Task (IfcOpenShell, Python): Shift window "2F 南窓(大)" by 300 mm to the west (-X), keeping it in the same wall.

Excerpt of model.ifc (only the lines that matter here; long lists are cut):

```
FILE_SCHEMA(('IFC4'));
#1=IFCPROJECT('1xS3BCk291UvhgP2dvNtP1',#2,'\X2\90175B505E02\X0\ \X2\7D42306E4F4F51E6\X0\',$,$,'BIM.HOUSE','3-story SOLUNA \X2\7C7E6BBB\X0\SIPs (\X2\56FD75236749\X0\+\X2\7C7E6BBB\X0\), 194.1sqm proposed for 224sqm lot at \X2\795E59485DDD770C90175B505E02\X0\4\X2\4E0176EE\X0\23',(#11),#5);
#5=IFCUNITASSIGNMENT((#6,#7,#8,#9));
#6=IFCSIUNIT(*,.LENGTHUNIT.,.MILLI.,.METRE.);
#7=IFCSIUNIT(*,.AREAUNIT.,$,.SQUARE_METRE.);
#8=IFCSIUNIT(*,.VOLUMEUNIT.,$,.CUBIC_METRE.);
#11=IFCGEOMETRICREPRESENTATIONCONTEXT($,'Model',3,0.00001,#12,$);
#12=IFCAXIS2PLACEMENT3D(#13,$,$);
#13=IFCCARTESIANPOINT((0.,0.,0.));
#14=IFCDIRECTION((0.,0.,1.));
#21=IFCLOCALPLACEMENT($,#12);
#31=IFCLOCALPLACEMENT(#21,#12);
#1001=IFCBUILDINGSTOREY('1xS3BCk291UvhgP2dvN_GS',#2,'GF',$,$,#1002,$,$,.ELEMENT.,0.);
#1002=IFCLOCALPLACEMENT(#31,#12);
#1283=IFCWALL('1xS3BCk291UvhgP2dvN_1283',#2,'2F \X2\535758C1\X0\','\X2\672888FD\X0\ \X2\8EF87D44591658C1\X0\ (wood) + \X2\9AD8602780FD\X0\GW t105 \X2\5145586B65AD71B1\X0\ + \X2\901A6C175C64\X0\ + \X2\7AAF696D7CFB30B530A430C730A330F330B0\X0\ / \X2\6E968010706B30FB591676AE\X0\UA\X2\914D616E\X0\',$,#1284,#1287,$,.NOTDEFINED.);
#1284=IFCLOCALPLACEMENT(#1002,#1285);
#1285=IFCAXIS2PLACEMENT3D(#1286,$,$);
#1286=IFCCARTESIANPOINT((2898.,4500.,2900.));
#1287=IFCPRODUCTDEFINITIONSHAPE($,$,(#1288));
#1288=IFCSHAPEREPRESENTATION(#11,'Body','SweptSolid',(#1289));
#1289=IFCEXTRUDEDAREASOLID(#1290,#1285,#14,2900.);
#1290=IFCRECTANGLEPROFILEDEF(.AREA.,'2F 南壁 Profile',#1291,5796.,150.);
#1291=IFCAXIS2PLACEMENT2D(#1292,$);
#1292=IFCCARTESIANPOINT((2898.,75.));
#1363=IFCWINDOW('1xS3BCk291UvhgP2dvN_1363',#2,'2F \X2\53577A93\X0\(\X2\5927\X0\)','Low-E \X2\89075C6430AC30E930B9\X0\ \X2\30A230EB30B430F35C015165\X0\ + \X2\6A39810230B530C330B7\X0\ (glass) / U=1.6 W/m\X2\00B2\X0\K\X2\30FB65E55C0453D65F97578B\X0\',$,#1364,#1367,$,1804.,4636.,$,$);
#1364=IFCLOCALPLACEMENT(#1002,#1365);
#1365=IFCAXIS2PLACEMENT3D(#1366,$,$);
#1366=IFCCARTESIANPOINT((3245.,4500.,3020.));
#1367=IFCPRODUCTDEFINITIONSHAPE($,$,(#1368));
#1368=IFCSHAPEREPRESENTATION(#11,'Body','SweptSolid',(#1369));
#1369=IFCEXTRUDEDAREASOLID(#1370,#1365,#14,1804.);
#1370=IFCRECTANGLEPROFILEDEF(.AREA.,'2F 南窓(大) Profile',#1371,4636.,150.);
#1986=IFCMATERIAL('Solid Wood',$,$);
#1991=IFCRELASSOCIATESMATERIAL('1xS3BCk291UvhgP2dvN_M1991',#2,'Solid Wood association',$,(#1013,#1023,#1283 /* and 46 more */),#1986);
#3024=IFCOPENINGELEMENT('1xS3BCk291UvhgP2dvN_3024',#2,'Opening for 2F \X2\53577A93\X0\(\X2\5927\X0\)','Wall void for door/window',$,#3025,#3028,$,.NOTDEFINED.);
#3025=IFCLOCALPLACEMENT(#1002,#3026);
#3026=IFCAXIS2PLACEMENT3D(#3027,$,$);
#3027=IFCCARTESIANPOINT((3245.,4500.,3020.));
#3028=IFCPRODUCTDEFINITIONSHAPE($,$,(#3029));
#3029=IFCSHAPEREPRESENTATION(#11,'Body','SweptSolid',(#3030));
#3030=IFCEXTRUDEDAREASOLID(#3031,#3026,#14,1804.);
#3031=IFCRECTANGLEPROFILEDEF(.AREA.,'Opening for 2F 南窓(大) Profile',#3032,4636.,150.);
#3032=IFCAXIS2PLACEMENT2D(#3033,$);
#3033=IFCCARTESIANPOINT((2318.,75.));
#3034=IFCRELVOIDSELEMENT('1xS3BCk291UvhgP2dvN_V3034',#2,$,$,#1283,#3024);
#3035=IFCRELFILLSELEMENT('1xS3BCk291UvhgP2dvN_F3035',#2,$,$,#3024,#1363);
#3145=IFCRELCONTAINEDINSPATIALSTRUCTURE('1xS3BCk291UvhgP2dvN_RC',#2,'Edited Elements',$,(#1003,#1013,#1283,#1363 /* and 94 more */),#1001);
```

```python
import ifcopenshell
import ifcopenshell.api.geometry
import ifcopenshell.util.placement

model = ifcopenshell.open("model.ifc")

window = model.by_guid("1xS3BCk291UvhgP2dvN_1363")
opening = window.FillsVoids[0].RelatingOpeningElement
wall = opening.VoidsElements[0].RelatingBuildingElement

wall_matrix = ifcopenshell.util.placement.get_local_placement(wall.ObjectPlacement)
shift = wall_matrix[:3, 0] * -300.0
before = ifcopenshell.util.placement.get_local_placement(window.ObjectPlacement)[:3, 3].copy()

# The window is not placed relative to its opening, so move both.
for product in (opening, window):
    matrix = ifcopenshell.util.placement.get_local_placement(product.ObjectPlacement)
    matrix[:3, 3] += shift
    ifcopenshell.api.geometry.edit_object_placement(model, product=product, matrix=matrix, is_si=False)

after = ifcopenshell.util.placement.get_local_placement(window.ObjectPlacement)[:3, 3]
print("window moved by", (after - before).round(3) + 0.0)

model.write("model-out.ifc")
```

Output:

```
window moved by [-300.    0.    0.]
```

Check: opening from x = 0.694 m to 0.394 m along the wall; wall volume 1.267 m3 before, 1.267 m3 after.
